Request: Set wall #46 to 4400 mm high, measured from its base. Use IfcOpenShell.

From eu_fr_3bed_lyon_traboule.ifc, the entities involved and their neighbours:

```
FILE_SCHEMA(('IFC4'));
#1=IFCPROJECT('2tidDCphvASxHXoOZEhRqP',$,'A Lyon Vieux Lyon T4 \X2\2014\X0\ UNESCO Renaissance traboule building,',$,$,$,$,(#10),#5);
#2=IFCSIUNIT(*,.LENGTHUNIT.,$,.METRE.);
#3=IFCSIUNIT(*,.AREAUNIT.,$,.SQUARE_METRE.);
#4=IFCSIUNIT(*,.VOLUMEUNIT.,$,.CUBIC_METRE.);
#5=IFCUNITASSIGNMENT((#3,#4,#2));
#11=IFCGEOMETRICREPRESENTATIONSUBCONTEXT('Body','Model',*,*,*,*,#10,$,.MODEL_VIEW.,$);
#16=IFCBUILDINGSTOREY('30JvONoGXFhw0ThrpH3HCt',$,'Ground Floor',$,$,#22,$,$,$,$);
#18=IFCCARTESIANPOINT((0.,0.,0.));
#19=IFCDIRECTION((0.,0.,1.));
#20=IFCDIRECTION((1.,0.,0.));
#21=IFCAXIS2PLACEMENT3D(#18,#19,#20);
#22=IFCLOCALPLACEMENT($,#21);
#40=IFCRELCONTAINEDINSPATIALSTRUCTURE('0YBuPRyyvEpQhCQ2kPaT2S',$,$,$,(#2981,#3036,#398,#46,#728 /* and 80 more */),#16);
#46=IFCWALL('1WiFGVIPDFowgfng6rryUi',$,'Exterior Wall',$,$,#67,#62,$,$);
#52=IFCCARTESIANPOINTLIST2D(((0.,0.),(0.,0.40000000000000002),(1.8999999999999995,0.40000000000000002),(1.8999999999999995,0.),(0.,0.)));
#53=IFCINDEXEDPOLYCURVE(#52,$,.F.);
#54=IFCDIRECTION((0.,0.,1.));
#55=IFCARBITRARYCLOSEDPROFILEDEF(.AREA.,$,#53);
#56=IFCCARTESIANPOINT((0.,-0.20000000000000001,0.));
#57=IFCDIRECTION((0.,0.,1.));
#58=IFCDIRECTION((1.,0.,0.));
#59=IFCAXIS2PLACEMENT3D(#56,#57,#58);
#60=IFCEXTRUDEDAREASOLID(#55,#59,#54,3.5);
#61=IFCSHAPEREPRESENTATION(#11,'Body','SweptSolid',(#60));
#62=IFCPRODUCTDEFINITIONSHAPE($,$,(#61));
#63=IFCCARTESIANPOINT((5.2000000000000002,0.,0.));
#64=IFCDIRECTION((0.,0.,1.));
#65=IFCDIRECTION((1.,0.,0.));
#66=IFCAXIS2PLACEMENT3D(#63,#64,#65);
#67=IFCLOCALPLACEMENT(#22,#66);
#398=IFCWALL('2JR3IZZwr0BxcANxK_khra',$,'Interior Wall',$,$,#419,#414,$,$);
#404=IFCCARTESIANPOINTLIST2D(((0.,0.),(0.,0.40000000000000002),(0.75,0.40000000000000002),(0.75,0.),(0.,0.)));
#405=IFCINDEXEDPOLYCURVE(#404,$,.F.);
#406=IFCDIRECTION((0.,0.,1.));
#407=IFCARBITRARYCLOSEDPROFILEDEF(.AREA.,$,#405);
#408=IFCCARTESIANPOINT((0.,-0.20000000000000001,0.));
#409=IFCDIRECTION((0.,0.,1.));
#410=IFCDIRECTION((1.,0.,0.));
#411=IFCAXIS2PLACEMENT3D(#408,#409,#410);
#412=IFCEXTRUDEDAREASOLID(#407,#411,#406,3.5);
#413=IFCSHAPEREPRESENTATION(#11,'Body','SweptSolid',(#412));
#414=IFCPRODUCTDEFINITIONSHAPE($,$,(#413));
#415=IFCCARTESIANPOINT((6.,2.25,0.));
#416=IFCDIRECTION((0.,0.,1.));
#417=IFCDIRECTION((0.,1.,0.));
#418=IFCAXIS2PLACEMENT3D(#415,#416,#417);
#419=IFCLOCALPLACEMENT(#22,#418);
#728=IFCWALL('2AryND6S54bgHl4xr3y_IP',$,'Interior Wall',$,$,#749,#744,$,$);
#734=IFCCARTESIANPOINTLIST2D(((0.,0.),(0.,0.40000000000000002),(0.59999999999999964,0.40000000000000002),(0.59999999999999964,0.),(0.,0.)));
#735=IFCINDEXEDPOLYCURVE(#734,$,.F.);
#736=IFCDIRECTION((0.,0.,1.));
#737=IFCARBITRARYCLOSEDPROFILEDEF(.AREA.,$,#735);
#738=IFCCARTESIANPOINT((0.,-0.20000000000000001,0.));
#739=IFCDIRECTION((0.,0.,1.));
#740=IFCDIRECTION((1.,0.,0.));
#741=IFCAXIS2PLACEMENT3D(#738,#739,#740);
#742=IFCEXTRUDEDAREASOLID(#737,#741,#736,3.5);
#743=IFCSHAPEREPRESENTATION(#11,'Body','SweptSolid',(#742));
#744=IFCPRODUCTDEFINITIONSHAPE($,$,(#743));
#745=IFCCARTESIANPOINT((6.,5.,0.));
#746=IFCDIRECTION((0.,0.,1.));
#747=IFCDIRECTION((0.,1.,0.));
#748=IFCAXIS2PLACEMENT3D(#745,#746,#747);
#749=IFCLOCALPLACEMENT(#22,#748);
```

```python
import ifcopenshell
import ifcopenshell.geom
import ifcopenshell.util.representation
import ifcopenshell.util.shape
import ifcopenshell.util.unit

model = ifcopenshell.open("eu_fr_3bed_lyon_traboule.ifc")
unit_scale = ifcopenshell.util.unit.calculate_unit_scale(model)
settings = ifcopenshell.geom.settings()


def volume(element):
    """Net volume in cubic metres, openings subtracted."""
    shape = ifcopenshell.geom.create_shape(settings, element)
    return ifcopenshell.util.shape.get_volume(shape.geometry)


wall = model.by_guid("1WiFGVIPDFowgfng6rryUi")
before = volume(wall)

body = ifcopenshell.util.representation.get_representation(wall, "Model", "Body")
solid = body.Items[0]
old_height = solid.Depth
solid.Depth = 4.4 / unit_scale
after = volume(wall)

print(f"height {old_height:g} -> {solid.Depth:g}, volume {before:.3f} -> {after:.3f} m3")

model.write("eu_fr_3bed_lyon_traboule_rev.ifc")
```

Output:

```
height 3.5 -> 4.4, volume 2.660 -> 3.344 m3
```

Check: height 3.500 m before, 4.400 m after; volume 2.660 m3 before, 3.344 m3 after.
